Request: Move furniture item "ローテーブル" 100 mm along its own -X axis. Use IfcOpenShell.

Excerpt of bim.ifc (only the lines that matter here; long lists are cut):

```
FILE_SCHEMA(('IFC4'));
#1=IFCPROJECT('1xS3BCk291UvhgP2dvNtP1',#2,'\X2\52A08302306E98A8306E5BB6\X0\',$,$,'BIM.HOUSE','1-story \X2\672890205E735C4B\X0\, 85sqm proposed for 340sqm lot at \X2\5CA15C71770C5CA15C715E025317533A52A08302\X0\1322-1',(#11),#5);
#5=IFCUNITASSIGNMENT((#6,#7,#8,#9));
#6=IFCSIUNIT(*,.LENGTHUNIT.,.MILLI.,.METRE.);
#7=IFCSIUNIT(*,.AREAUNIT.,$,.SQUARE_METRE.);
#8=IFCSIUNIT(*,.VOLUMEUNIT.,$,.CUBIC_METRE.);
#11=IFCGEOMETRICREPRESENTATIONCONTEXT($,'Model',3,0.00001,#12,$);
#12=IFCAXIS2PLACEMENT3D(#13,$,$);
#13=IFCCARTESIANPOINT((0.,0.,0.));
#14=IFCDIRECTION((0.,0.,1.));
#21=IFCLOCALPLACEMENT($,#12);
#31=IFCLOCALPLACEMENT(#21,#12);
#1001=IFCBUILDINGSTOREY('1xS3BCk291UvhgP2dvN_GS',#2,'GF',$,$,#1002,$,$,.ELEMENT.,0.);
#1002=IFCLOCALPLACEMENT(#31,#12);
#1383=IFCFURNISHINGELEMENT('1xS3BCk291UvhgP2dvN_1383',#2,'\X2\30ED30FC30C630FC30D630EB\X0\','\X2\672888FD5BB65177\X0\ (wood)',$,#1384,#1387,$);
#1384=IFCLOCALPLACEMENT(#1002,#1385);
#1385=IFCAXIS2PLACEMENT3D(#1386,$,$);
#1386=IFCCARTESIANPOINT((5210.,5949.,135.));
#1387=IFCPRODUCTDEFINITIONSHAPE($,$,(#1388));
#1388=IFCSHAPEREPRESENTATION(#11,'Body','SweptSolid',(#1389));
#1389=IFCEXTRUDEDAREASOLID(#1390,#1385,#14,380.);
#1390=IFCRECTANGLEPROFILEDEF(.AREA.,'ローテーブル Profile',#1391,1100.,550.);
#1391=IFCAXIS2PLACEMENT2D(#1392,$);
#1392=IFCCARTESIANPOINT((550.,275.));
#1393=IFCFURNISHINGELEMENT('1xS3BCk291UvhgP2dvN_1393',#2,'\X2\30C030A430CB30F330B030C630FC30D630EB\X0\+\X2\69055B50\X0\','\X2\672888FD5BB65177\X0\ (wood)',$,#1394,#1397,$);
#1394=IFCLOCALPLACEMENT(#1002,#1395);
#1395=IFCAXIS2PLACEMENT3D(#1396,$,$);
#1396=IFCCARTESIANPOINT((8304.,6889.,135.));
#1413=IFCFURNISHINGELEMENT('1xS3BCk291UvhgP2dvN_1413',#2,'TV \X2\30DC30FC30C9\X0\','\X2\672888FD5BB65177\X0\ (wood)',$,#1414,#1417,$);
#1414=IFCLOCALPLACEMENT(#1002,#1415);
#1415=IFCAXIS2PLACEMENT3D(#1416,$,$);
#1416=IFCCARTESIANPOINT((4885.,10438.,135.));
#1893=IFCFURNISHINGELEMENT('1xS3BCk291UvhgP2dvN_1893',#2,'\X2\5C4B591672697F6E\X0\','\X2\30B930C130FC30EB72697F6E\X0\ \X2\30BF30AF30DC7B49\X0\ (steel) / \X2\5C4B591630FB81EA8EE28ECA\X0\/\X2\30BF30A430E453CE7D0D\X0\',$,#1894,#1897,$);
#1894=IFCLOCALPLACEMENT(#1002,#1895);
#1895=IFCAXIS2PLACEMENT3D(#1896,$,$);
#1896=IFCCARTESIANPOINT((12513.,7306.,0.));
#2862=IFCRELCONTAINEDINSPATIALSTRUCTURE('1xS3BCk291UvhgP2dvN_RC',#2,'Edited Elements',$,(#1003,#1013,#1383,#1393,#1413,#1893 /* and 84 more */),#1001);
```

```python
import ifcopenshell
import ifcopenshell.api.geometry
import ifcopenshell.util.placement

model = ifcopenshell.open("bim.ifc")

item = model.by_guid("1xS3BCk291UvhgP2dvN_1383")
matrix = ifcopenshell.util.placement.get_local_placement(item.ObjectPlacement)
matrix[:3, 3] -= matrix[:3, 0] * 100.0
ifcopenshell.api.geometry.edit_object_placement(model, product=item, matrix=matrix, is_si=False)

print(ifcopenshell.util.placement.get_local_placement(item.ObjectPlacement).round(3) + 0.0)

model.write("bim_edited.ifc")
```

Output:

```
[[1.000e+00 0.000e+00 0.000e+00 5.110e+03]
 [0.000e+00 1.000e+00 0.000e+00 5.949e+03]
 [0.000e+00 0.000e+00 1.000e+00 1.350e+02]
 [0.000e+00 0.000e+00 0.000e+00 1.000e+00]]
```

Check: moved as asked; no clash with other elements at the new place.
